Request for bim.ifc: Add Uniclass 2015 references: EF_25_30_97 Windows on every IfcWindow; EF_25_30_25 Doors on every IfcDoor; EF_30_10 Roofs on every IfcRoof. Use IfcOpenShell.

First a look at what the model holds.

```python
import ifcopenshell

model = ifcopenshell.open("bim.ifc")
print(model.schema)
print("classifications:", [c.Name for c in model.by_type("IfcClassification")])
for ifc_class in ("IfcDoor", "IfcRoof", "IfcStair", "IfcWall", "IfcWindow"):
    print(ifc_class, len(model.by_type(ifc_class)))
```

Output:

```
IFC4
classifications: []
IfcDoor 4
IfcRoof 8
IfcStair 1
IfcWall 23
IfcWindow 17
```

```python
import ifcopenshell
import ifcopenshell.api.classification

model = ifcopenshell.open("bim.ifc")

system = ifcopenshell.api.classification.add_classification(model, classification="Uniclass 2015")

codes = {
    "IfcWindow": ("EF_25_30_97", "Windows"),
    "IfcDoor": ("EF_25_30_25", "Doors"),
    "IfcRoof": ("EF_30_10", "Roofs"),
}
for ifc_class, (code, name) in codes.items():
    products = model.by_type(ifc_class)
    ifcopenshell.api.classification.add_reference(
        model, products=products, classification=system, identification=code, name=name
    )
    print(code, len(products))

model.write("bim_rev.ifc")
```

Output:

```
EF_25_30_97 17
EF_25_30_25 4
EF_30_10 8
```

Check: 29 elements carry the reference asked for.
